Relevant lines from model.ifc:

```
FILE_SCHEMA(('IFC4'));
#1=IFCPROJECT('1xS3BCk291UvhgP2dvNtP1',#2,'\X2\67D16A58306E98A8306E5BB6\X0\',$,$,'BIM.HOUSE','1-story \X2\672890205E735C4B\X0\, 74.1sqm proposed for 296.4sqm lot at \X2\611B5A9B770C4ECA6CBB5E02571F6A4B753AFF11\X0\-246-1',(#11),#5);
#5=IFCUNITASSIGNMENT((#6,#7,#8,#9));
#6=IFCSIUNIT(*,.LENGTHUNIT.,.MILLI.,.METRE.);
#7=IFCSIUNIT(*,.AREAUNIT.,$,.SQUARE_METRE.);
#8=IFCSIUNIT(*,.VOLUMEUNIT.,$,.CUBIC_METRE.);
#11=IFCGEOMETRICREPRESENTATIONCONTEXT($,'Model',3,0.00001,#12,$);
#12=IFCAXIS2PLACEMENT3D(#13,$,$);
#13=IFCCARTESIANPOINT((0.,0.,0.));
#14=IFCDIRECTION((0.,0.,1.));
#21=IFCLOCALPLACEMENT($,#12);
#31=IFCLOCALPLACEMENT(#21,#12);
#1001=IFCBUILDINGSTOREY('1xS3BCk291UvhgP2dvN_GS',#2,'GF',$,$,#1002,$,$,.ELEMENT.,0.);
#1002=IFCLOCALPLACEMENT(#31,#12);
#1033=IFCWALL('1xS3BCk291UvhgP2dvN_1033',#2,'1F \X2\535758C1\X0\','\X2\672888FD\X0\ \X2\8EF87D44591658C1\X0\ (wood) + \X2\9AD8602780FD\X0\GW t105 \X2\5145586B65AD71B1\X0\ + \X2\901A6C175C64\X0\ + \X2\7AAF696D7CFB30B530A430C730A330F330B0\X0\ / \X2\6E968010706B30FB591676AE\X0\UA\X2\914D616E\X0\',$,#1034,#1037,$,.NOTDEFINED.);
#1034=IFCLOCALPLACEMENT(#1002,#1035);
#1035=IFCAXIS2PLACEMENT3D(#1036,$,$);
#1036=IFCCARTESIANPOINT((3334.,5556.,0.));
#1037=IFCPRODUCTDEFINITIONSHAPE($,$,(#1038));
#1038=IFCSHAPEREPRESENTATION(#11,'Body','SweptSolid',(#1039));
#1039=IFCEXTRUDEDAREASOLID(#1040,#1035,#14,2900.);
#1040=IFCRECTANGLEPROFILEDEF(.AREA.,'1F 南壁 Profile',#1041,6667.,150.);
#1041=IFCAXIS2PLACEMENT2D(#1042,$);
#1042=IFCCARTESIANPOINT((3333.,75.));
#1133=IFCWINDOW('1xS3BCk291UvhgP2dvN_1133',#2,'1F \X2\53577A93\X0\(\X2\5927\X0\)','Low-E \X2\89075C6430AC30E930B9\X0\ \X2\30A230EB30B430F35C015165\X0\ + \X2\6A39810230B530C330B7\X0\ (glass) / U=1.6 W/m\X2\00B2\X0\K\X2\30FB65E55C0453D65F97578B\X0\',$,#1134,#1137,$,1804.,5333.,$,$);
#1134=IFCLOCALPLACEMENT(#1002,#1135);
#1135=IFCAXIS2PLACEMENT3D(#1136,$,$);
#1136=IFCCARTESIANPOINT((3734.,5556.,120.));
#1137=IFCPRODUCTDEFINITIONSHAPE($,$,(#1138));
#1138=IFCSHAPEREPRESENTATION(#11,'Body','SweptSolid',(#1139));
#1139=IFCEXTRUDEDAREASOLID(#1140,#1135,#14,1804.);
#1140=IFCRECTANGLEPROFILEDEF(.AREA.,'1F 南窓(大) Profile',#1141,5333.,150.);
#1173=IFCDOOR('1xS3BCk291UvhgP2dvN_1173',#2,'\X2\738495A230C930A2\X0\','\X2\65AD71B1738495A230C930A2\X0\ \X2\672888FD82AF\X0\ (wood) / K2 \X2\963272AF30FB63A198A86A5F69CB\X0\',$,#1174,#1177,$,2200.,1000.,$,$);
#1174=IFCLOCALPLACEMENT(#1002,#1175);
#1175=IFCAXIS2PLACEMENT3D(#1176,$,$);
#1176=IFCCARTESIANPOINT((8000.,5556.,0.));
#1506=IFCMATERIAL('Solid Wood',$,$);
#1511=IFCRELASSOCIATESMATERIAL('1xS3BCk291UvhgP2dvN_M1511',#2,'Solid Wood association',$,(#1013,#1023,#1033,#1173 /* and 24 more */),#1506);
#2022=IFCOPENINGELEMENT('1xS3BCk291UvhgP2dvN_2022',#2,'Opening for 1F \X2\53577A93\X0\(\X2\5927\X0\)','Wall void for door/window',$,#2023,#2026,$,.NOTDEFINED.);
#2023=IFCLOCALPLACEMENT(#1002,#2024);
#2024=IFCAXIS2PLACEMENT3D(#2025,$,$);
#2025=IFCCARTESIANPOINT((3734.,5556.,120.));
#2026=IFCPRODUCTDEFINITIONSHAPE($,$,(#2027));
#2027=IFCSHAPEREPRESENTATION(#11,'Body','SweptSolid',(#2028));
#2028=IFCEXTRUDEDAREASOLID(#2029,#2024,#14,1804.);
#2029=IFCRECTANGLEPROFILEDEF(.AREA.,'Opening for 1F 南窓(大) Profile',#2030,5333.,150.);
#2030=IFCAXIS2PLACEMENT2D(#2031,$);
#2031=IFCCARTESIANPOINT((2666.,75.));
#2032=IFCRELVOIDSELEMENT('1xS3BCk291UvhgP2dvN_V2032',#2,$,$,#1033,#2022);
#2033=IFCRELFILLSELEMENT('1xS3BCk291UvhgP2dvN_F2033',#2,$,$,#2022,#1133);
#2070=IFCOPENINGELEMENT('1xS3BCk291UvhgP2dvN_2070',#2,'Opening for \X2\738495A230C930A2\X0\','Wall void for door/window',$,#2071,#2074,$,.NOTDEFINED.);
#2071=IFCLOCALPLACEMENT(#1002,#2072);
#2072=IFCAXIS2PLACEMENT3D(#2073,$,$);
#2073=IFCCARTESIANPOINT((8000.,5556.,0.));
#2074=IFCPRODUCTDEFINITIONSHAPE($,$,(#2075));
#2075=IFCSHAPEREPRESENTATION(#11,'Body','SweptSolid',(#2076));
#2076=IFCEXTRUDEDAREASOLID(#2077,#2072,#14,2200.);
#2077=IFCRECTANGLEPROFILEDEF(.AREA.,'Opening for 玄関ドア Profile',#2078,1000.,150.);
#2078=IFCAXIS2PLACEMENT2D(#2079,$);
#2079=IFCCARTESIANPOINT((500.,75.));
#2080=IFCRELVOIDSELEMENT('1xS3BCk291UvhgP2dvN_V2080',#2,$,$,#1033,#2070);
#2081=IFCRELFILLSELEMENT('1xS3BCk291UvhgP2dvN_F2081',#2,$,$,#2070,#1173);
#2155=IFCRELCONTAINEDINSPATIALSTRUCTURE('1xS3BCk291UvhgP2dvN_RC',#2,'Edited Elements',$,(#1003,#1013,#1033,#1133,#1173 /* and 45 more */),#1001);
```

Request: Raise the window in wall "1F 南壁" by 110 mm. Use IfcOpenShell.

```python
import numpy as np
import ifcopenshell
import ifcopenshell.api.geometry
import ifcopenshell.util.placement
import ifcopenshell.util.unit

model = ifcopenshell.open("model.ifc")
unit_scale = ifcopenshell.util.unit.calculate_unit_scale(model)

window = model.by_guid("1xS3BCk291UvhgP2dvN_1133")
opening = window.FillsVoids[0].RelatingOpeningElement
dz = 0.11 / unit_scale

shift = np.array([0.0, 0.0, dz])
# The window is not placed relative to its opening, so move both.
for product in (opening, window):
    matrix = ifcopenshell.util.placement.get_local_placement(product.ObjectPlacement)
    matrix[:3, 3] += shift
    ifcopenshell.api.geometry.edit_object_placement(model, product=product, matrix=matrix, is_si=False)

print(f"moved by {dz * unit_scale:+.3f} m")

model.write("model_v2.ifc")
```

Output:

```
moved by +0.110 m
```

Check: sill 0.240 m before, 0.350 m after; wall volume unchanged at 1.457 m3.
